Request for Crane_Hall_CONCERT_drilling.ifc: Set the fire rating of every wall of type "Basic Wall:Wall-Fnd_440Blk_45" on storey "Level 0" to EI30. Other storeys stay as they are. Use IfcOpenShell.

First a look at what the model holds.

```python
import ifcopenshell
import ifcopenshell.util.element

model = ifcopenshell.open("Crane_Hall_CONCERT_drilling.ifc")
print(model.schema)
storey = next(s for s in model.by_type("IfcBuildingStorey") if s.Name == "Level 0")
walls = [e for e in ifcopenshell.util.element.get_decomposition(storey) if e.is_a("IfcWall")]
seen = {}
for e in walls:
    element_type = ifcopenshell.util.element.get_type(e)
    key = (element_type.Name if element_type != e and element_type else None, ifcopenshell.util.element.get_pset(e, "Pset_WallCommon", "FireRating"))
    seen[key] = seen.get(key, 0) + 1
for (name, value), count in sorted(seen.items(), key=str):
    print(count, "x", name, "|", value)
```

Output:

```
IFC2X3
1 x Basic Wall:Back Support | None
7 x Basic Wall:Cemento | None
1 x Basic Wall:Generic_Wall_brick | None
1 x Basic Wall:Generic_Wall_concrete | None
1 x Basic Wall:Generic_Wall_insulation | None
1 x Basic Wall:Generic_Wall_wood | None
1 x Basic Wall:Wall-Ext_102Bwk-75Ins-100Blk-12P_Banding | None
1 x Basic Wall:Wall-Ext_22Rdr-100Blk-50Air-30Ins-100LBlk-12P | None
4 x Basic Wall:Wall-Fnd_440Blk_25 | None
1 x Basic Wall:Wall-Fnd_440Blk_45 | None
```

```python
import ifcopenshell
import ifcopenshell.api.pset
import ifcopenshell.util.element

model = ifcopenshell.open("Crane_Hall_CONCERT_drilling.ifc")

storey = next(s for s in model.by_type("IfcBuildingStorey") if s.Name == "Level 0")
walls = [e for e in ifcopenshell.util.element.get_decomposition(storey) if e.is_a("IfcWall")]

count = 0
for e in walls:
    element_type = ifcopenshell.util.element.get_type(e)
    if element_type in (None, e) or element_type.Name != "Basic Wall:Wall-Fnd_440Blk_45":
        continue
    # add_pset returns the element's existing set when there is one.
    pset = ifcopenshell.api.pset.add_pset(model, product=e, name="Pset_WallCommon")
    ifcopenshell.api.pset.edit_pset(model, pset=pset, properties={"FireRating": "EI30"})
    count += 1

print(count, "walls updated")

model.write("Crane_Hall_CONCERT_drilling_updated.ifc")
```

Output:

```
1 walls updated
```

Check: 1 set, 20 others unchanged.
